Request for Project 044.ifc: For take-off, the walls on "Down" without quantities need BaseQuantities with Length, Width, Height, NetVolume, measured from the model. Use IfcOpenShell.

First a look at what the model holds.

```python
import ifcopenshell
import ifcopenshell.util.element
import ifcopenshell.util.unit

model = ifcopenshell.open("Project 044.ifc")
print(model.schema)
for unit_type in ("LENGTHUNIT", "AREAUNIT", "VOLUMEUNIT"):
    print(unit_type, ifcopenshell.util.unit.calculate_unit_scale(model, unit_type))
storey = next(s for s in model.by_type("IfcBuildingStorey") if s.Name == "Down")
walls = [e for e in ifcopenshell.util.element.get_decomposition(storey) if e.is_a("IfcWall")]
for e in sorted(walls, key=lambda e: e.id()):
    print(e.id(), e.is_a(), e.Name, list(ifcopenshell.util.element.get_psets(e, qtos_only=True)), sep=" | ")
```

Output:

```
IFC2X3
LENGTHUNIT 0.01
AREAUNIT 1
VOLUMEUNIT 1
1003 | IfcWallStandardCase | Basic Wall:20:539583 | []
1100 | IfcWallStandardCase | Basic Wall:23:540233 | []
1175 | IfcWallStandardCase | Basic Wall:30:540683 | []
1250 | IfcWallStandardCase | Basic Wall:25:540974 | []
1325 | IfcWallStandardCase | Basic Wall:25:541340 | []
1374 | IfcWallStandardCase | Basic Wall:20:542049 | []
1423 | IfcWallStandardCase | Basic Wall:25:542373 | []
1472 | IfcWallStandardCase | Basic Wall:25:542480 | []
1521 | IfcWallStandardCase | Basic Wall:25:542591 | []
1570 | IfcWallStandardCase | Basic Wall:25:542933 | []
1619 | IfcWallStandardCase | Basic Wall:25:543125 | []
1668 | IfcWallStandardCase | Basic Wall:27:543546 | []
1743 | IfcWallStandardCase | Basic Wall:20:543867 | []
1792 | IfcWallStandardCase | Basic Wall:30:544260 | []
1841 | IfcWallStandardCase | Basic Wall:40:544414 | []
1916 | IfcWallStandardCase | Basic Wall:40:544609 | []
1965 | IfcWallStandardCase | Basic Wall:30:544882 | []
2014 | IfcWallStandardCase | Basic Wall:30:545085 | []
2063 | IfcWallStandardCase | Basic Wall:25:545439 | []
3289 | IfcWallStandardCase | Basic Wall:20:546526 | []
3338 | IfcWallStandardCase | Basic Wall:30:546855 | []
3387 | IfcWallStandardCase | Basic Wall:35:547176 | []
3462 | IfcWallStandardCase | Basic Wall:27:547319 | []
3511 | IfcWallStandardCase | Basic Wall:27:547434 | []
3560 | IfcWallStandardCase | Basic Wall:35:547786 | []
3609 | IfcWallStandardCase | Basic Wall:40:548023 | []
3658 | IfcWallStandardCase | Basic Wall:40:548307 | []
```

```python
import ifcopenshell
import ifcopenshell.api.pset
import ifcopenshell.geom
import ifcopenshell.util.element
import ifcopenshell.util.shape
import ifcopenshell.util.unit

model = ifcopenshell.open("Project 044.ifc")
unit_scale = ifcopenshell.util.unit.calculate_unit_scale(model)
volume_scale = ifcopenshell.util.unit.calculate_unit_scale(model, "VOLUMEUNIT")
settings = ifcopenshell.geom.settings()

storey = next(s for s in model.by_type("IfcBuildingStorey") if s.Name == "Down")
walls = [e for e in ifcopenshell.util.element.get_decomposition(storey) if e.is_a("IfcWall")]

for e in sorted(walls, key=lambda e: e.id()):
    if ifcopenshell.util.element.get_psets(e, qtos_only=True, should_inherit=False):
        continue
    # Geometry comes back in metres, in the element's own axes.
    shape = ifcopenshell.geom.create_shape(settings, e)
    values = {
        "Length": ifcopenshell.util.shape.get_x(shape.geometry) / unit_scale,
        "Width": ifcopenshell.util.shape.get_y(shape.geometry) / unit_scale,
        "Height": ifcopenshell.util.shape.get_z(shape.geometry) / unit_scale,
        "NetVolume": ifcopenshell.util.shape.get_volume(shape.geometry) / volume_scale,
    }
    qto = ifcopenshell.api.pset.add_qto(model, product=e, name="BaseQuantities")
    ifcopenshell.api.pset.edit_qto(model, qto=qto, properties=values)
    print(e.id(), {k: round(v, 3) for k, v in values.items()})

model.write("Project 044_edited.ifc")
```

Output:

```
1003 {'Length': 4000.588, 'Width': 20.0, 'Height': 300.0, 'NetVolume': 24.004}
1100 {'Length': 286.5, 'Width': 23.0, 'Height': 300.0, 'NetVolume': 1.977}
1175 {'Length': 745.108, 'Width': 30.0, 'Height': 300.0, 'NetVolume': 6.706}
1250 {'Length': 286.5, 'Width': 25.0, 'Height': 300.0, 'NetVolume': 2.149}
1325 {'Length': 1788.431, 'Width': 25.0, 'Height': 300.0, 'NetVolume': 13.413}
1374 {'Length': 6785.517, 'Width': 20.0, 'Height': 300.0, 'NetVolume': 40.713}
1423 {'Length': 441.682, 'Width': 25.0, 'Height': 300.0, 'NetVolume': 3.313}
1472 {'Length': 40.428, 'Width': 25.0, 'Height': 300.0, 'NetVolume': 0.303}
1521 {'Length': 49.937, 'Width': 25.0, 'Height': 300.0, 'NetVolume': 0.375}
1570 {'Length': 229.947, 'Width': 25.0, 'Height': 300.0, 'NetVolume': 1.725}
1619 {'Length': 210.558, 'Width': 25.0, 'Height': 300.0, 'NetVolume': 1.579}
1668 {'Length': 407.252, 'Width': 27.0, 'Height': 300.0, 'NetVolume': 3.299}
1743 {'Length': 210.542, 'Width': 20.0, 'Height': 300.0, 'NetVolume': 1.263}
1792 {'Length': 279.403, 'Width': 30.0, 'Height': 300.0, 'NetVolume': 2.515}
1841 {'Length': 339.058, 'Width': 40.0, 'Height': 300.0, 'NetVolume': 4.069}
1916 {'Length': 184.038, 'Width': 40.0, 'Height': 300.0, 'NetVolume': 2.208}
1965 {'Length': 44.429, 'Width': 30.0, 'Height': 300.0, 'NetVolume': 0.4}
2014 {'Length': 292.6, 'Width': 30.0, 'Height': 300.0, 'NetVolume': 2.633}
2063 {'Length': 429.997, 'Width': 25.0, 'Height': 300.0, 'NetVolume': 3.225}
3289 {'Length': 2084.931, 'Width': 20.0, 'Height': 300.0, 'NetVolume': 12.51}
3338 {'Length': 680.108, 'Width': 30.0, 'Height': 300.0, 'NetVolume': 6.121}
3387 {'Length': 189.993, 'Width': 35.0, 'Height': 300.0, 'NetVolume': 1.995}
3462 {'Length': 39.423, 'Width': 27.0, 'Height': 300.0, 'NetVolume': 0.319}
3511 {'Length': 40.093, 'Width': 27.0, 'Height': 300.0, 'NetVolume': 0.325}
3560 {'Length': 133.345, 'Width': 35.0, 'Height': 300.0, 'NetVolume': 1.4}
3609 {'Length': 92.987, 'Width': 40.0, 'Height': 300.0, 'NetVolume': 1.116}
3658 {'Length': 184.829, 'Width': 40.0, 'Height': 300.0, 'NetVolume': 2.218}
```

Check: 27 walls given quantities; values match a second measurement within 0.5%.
